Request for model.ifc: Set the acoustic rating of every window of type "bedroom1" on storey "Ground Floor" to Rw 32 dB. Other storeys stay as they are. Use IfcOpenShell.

First a look at what the model holds.

```python
import ifcopenshell
import ifcopenshell.util.element

model = ifcopenshell.open("model.ifc")
print(model.schema)
storey = next(s for s in model.by_type("IfcBuildingStorey") if s.Name == "Ground Floor")
windows = [e for e in ifcopenshell.util.element.get_decomposition(storey) if e.is_a("IfcWindow")]
seen = {}
for e in windows:
    element_type = ifcopenshell.util.element.get_type(e)
    key = (element_type.Name if element_type != e and element_type else None, ifcopenshell.util.element.get_pset(e, "Pset_WindowCommon", "AcousticRating"))
    seen[key] = seen.get(key, 0) + 1
for (name, value), count in sorted(seen.items(), key=str):
    print(count, "x", name, "|", value)
```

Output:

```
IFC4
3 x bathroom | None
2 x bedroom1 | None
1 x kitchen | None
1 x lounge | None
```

```python
import ifcopenshell
import ifcopenshell.api.pset
import ifcopenshell.util.element

model = ifcopenshell.open("model.ifc")

storey = next(s for s in model.by_type("IfcBuildingStorey") if s.Name == "Ground Floor")
windows = [e for e in ifcopenshell.util.element.get_decomposition(storey) if e.is_a("IfcWindow")]

count = 0
for e in windows:
    element_type = ifcopenshell.util.element.get_type(e)
    if element_type in (None, e) or element_type.Name != "bedroom1":
        continue
    # add_pset returns the element's existing set when there is one.
    pset = ifcopenshell.api.pset.add_pset(model, product=e, name="Pset_WindowCommon")
    ifcopenshell.api.pset.edit_pset(model, pset=pset, properties={"AcousticRating": "Rw 32 dB"})
    count += 1

print(count, "windows updated")

model.write("model-out.ifc")
```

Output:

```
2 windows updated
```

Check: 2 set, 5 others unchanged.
